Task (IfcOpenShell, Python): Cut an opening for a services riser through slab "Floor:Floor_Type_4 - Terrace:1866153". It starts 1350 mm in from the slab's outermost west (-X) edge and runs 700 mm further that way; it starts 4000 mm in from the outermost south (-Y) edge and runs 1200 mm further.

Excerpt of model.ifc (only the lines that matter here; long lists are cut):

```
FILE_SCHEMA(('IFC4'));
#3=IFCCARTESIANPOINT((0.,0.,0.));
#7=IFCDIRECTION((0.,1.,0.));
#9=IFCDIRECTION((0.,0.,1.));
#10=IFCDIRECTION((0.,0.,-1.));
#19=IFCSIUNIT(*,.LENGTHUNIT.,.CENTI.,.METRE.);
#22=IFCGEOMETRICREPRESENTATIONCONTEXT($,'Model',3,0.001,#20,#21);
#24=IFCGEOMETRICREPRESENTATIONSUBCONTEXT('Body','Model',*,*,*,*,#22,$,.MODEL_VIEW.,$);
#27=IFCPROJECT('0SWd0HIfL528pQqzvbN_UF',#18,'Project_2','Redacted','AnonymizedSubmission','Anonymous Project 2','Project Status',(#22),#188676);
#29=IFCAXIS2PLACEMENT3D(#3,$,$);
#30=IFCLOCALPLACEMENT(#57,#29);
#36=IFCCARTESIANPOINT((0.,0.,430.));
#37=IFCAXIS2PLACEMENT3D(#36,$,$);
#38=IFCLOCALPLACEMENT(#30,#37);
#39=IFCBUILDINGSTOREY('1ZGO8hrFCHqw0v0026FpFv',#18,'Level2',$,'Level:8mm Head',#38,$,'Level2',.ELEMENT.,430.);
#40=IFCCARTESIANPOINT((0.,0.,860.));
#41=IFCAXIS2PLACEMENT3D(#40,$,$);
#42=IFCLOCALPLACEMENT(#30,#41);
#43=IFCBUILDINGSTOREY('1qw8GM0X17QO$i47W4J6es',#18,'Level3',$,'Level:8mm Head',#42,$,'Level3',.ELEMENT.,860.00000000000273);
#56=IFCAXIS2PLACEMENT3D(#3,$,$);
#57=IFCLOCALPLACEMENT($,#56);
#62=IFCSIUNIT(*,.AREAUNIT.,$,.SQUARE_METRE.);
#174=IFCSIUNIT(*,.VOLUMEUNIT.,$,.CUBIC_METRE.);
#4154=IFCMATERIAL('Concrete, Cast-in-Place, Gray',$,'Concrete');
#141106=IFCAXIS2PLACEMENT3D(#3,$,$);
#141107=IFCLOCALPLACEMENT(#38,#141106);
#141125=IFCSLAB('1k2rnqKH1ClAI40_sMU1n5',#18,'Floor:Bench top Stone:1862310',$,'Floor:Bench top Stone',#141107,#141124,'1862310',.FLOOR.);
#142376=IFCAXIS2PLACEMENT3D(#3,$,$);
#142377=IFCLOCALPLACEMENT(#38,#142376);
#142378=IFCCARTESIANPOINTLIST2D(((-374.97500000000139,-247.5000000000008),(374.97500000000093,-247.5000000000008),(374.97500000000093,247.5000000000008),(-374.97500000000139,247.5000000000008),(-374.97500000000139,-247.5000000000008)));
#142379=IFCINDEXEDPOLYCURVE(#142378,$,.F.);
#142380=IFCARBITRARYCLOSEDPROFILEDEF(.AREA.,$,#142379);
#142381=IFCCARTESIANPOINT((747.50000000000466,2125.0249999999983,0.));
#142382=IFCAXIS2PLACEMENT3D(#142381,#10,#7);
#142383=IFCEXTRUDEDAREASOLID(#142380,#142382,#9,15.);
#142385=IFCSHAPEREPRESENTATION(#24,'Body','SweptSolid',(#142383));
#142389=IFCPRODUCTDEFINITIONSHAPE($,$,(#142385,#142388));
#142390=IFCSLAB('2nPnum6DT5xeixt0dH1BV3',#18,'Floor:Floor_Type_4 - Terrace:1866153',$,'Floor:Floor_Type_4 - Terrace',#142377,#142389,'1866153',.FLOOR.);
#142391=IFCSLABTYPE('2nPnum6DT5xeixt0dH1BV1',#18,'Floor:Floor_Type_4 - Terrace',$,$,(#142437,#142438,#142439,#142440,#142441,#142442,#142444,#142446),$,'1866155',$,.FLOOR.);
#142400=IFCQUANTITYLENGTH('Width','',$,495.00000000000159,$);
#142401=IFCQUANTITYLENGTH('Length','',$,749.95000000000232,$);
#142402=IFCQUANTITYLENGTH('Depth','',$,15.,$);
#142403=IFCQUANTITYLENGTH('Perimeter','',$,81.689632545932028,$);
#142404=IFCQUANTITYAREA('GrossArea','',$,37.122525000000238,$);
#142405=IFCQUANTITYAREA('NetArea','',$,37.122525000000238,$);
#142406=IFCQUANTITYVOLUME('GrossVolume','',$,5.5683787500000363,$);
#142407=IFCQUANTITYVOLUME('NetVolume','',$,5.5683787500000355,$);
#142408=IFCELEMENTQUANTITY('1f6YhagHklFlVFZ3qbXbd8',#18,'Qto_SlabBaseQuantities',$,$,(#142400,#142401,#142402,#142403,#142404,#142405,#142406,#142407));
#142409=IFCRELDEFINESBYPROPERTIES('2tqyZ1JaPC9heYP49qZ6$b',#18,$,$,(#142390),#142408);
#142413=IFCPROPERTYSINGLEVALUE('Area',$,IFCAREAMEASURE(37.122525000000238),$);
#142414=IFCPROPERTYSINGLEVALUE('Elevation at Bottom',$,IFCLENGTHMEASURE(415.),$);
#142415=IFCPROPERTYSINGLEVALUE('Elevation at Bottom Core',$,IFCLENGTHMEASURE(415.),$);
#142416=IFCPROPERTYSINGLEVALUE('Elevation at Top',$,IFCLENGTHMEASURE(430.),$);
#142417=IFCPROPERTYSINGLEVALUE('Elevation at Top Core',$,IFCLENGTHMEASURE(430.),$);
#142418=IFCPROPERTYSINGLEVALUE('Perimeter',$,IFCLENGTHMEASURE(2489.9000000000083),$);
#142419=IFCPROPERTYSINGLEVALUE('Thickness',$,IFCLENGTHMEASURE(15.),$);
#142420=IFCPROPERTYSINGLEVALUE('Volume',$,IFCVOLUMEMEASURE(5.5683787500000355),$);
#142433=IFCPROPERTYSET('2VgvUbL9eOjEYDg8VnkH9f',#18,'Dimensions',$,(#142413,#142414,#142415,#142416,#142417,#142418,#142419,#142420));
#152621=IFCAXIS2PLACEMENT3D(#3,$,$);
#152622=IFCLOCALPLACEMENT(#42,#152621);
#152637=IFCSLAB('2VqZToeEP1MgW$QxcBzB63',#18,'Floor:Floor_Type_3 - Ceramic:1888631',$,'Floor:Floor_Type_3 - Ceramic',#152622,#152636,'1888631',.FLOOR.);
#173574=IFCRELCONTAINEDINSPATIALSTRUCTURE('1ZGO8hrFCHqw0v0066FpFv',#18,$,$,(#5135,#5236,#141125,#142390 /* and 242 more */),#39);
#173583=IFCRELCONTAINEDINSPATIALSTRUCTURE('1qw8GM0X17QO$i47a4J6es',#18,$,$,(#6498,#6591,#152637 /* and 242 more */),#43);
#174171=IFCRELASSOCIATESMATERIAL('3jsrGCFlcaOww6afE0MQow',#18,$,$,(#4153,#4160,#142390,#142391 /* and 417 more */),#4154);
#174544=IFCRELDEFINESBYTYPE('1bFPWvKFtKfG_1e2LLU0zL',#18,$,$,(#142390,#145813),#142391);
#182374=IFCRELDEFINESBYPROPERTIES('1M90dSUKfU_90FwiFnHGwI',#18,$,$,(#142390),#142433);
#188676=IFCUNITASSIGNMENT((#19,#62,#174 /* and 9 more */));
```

```python
import numpy as np
import ifcopenshell
import ifcopenshell.api.feature
import ifcopenshell.api.geometry
import ifcopenshell.api.pset
import ifcopenshell.api.root
import ifcopenshell.geom
import ifcopenshell.util.element
import ifcopenshell.util.placement
import ifcopenshell.util.representation
import ifcopenshell.util.shape
import ifcopenshell.util.unit

model = ifcopenshell.open("model.ifc")
unit_scale = ifcopenshell.util.unit.calculate_unit_scale(model)
area_scale = ifcopenshell.util.unit.calculate_unit_scale(model, "AREAUNIT")
volume_scale = ifcopenshell.util.unit.calculate_unit_scale(model, "VOLUMEUNIT")
settings = ifcopenshell.geom.settings()


def volume(element):
    """Net volume in cubic metres, openings subtracted."""
    shape = ifcopenshell.geom.create_shape(settings, element)
    return ifcopenshell.util.shape.get_volume(shape.geometry)


slab = model.by_id(142390)
before = volume(slab)

# Extent in the slab's own axes, in metres. The edges named are its -X and -Y sides.
slab_shape = ifcopenshell.geom.create_shape(settings, slab)
vertices = ifcopenshell.util.shape.get_vertices(slab_shape.geometry)
x_min, y_min, bottom = vertices.min(axis=0)
top = vertices[:, 2].max()

opening = ifcopenshell.api.root.create_entity(model, ifc_class="IfcOpeningElement", name="Services riser opening", predefined_type="OPENING")
context = ifcopenshell.util.representation.get_context(model, "Model", "Body", "MODEL_VIEW")
width, depth = 0.7, 1.2
outline = [(0.0, 0.0), (width, 0.0), (width, depth), (0.0, depth), (0.0, 0.0)]
# Overshoot both faces by 50 mm so the cut is clean.
shape = ifcopenshell.api.geometry.add_slab_representation(
    model, context=context, depth=top - bottom + 0.1, polyline=outline
)
ifcopenshell.api.geometry.assign_representation(model, product=opening, representation=shape)

matrix = ifcopenshell.util.placement.get_local_placement(slab.ObjectPlacement)
matrix[:, 3] = matrix @ np.append(np.array([x_min + 1.35, y_min + 4, bottom - 0.05]) / unit_scale, 1.0)
ifcopenshell.api.geometry.edit_object_placement(model, product=opening, matrix=matrix, is_si=False)
ifcopenshell.api.feature.add_feature(model, feature=opening, element=slab)

after = volume(slab)

# Update the slab's stored quantities.
qto = model.by_id(ifcopenshell.util.element.get_pset(slab, "Qto_SlabBaseQuantities", should_inherit=False)["id"])
ifcopenshell.api.pset.edit_qto(model, qto=qto, properties={
    "NetArea": after / (top - bottom) / area_scale,
    "NetVolume": after / volume_scale,
})
pset = model.by_id(ifcopenshell.util.element.get_pset(slab, "Dimensions", should_inherit=False)["id"])
ifcopenshell.api.pset.edit_pset(model, pset=pset, properties={
    "Area": model.create_entity("IfcAreaMeasure", after / (top - bottom) / area_scale),
    "Volume": model.create_entity("IfcVolumeMeasure", after / volume_scale),
})

print(f"slab volume {before:.3f} -> {after:.3f} m3")

model.write("model_rev.ifc")
```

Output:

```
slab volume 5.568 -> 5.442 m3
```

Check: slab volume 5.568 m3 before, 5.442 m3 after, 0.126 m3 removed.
